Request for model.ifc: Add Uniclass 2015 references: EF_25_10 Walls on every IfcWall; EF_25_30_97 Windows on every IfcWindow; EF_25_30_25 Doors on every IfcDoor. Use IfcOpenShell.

First a look at what the model holds.

```python
import ifcopenshell

model = ifcopenshell.open("model.ifc")
print(model.schema)
print("classifications:", [c.Name for c in model.by_type("IfcClassification")])
for ifc_class in ("IfcDoor", "IfcRoof", "IfcStair", "IfcWall", "IfcWindow"):
    print(ifc_class, len(model.by_type(ifc_class)))
```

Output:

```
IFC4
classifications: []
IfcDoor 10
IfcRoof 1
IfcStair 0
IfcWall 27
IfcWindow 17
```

```python
import ifcopenshell
import ifcopenshell.api.classification

model = ifcopenshell.open("model.ifc")

system = ifcopenshell.api.classification.add_classification(model, classification="Uniclass 2015")

codes = {
    "IfcWall": ("EF_25_10", "Walls"),
    "IfcWindow": ("EF_25_30_97", "Windows"),
    "IfcDoor": ("EF_25_30_25", "Doors"),
}
for ifc_class, (code, name) in codes.items():
    products = model.by_type(ifc_class)
    ifcopenshell.api.classification.add_reference(
        model, products=products, classification=system, identification=code, name=name
    )
    print(code, len(products))

model.write("model_rev.ifc")
```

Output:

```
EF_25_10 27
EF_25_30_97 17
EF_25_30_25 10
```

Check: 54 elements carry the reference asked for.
